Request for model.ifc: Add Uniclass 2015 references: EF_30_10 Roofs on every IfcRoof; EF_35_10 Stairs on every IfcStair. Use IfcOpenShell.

First a look at what the model holds.

```python
import ifcopenshell

model = ifcopenshell.open("model.ifc")
print(model.schema)
print("classifications:", [c.Name for c in model.by_type("IfcClassification")])
for ifc_class in ("IfcDoor", "IfcRoof", "IfcStair", "IfcWall", "IfcWindow"):
    print(ifc_class, len(model.by_type(ifc_class)))
```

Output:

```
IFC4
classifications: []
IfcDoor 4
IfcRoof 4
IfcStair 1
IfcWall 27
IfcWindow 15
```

```python
import ifcopenshell
import ifcopenshell.api.classification

model = ifcopenshell.open("model.ifc")

system = ifcopenshell.api.classification.add_classification(model, classification="Uniclass 2015")

codes = {
    "IfcRoof": ("EF_30_10", "Roofs"),
    "IfcStair": ("EF_35_10", "Stairs"),
}
for ifc_class, (code, name) in codes.items():
    products = model.by_type(ifc_class)
    ifcopenshell.api.classification.add_reference(
        model, products=products, classification=system, identification=code, name=name
    )
    print(code, len(products))

model.write("model_edited.ifc")
```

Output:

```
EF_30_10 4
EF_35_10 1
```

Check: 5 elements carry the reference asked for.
